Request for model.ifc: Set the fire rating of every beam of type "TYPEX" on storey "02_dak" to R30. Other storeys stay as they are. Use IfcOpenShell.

First a look at what the model holds.

```python
import ifcopenshell
import ifcopenshell.util.element

model = ifcopenshell.open("model.ifc")
print(model.schema)
storey = next(s for s in model.by_type("IfcBuildingStorey") if s.Name == "02_dak")
beams = [e for e in ifcopenshell.util.element.get_decomposition(storey) if e.is_a("IfcBeam")]
seen = {}
for e in beams:
    element_type = ifcopenshell.util.element.get_type(e)
    key = (element_type.Name if element_type != e and element_type else None, ifcopenshell.util.element.get_pset(e, "Pset_BeamCommon", "FireRating"))
    seen[key] = seen.get(key, 0) + 1
for (name, value), count in sorted(seen.items(), key=str):
    print(count, "x", name, "|", value)
```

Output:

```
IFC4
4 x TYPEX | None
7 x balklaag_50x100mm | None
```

```python
import ifcopenshell
import ifcopenshell.api.pset
import ifcopenshell.util.element

model = ifcopenshell.open("model.ifc")

storey = next(s for s in model.by_type("IfcBuildingStorey") if s.Name == "02_dak")
beams = [e for e in ifcopenshell.util.element.get_decomposition(storey) if e.is_a("IfcBeam")]

count = 0
for e in beams:
    element_type = ifcopenshell.util.element.get_type(e)
    if element_type in (None, e) or element_type.Name != "TYPEX":
        continue
    # add_pset returns the element's existing set when there is one.
    pset = ifcopenshell.api.pset.add_pset(model, product=e, name="Pset_BeamCommon")
    ifcopenshell.api.pset.edit_pset(model, pset=pset, properties={"FireRating": "R30"})
    count += 1

print(count, "beams updated")

model.write("model_rev.ifc")
```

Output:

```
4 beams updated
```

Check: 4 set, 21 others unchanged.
